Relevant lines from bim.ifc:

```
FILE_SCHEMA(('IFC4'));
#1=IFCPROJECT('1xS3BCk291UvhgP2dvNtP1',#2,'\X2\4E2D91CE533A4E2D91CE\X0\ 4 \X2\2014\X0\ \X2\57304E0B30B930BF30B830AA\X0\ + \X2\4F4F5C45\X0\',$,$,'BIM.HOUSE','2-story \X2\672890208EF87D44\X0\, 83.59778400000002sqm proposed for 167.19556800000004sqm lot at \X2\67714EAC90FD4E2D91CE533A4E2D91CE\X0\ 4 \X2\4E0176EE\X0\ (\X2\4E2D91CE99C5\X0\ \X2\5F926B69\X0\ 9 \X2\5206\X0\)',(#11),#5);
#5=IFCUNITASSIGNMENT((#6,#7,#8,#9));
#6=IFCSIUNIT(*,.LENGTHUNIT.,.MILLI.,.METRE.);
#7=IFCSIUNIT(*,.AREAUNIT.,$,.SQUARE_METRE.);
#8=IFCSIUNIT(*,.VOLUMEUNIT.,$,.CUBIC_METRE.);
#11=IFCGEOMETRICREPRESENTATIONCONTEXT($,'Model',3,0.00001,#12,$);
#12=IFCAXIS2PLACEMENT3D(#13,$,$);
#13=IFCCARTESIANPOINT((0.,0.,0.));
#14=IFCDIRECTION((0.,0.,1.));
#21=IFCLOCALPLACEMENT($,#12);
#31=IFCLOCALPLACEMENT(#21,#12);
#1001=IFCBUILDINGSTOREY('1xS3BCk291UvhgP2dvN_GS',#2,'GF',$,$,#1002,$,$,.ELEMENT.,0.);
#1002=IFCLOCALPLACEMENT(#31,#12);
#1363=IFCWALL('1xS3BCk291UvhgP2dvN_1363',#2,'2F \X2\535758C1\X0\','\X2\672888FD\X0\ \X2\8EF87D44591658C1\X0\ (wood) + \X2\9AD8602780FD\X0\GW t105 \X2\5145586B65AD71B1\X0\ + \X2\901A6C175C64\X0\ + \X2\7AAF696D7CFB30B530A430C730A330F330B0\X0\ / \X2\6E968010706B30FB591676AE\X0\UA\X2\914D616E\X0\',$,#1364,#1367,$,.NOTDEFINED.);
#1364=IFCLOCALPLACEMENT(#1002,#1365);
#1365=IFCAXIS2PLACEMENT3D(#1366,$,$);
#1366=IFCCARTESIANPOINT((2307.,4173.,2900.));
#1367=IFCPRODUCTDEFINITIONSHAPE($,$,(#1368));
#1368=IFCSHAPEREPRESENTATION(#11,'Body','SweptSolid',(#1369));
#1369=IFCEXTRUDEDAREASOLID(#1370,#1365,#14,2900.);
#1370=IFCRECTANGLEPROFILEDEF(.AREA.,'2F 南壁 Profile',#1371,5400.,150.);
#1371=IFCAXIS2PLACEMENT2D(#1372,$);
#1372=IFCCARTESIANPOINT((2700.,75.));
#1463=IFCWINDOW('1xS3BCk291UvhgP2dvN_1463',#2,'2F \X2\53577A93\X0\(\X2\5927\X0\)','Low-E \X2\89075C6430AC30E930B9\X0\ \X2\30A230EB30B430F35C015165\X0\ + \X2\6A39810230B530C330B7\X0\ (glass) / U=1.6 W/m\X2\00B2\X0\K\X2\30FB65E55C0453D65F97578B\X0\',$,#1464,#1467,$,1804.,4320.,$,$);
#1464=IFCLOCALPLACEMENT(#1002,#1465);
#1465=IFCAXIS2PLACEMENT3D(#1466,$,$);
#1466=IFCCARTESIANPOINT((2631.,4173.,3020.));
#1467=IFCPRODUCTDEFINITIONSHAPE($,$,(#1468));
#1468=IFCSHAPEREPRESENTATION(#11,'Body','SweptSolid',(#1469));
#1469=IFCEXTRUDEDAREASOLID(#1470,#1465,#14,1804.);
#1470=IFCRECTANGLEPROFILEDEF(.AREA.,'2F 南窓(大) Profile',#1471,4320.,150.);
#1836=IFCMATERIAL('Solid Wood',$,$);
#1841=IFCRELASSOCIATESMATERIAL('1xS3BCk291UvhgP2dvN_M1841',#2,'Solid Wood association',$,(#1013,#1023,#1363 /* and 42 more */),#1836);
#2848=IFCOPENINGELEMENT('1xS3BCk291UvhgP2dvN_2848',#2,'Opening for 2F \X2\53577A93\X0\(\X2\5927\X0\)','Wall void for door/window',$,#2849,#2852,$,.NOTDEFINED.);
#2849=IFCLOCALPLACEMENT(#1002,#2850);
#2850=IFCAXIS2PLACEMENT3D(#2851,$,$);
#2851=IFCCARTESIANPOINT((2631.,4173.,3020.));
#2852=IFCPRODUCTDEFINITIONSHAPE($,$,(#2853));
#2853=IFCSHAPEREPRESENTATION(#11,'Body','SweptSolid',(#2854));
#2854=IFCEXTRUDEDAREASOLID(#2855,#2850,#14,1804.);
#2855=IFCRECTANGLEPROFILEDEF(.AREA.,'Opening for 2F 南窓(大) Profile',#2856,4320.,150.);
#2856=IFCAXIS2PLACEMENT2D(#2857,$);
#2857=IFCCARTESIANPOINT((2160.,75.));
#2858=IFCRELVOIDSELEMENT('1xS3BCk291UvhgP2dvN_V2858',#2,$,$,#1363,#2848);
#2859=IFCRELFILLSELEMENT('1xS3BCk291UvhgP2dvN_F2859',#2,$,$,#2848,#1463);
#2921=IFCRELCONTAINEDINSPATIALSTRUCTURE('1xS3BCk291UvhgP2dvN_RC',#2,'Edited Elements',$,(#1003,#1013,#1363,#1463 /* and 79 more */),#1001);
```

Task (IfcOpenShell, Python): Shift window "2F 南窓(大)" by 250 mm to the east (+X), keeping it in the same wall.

```python
import ifcopenshell
import ifcopenshell.api.geometry
import ifcopenshell.util.placement
import ifcopenshell.util.unit

model = ifcopenshell.open("bim.ifc")
unit_scale = ifcopenshell.util.unit.calculate_unit_scale(model)

window = model.by_guid("1xS3BCk291UvhgP2dvN_1463")
opening = window.FillsVoids[0].RelatingOpeningElement
wall = opening.VoidsElements[0].RelatingBuildingElement

wall_matrix = ifcopenshell.util.placement.get_local_placement(wall.ObjectPlacement)
shift = wall_matrix[:3, 0] * 0.25 / unit_scale
before = ifcopenshell.util.placement.get_local_placement(window.ObjectPlacement)[:3, 3].copy()

# The window is not placed relative to its opening, so move both.
for product in (opening, window):
    matrix = ifcopenshell.util.placement.get_local_placement(product.ObjectPlacement)
    matrix[:3, 3] += shift
    ifcopenshell.api.geometry.edit_object_placement(model, product=product, matrix=matrix, is_si=False)

after = ifcopenshell.util.placement.get_local_placement(window.ObjectPlacement)[:3, 3]
print("window moved by", (after - before).round(3) + 0.0)

model.write("bim_v2.ifc")
```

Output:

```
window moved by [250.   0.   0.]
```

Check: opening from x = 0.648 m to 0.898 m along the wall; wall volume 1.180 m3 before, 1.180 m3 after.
